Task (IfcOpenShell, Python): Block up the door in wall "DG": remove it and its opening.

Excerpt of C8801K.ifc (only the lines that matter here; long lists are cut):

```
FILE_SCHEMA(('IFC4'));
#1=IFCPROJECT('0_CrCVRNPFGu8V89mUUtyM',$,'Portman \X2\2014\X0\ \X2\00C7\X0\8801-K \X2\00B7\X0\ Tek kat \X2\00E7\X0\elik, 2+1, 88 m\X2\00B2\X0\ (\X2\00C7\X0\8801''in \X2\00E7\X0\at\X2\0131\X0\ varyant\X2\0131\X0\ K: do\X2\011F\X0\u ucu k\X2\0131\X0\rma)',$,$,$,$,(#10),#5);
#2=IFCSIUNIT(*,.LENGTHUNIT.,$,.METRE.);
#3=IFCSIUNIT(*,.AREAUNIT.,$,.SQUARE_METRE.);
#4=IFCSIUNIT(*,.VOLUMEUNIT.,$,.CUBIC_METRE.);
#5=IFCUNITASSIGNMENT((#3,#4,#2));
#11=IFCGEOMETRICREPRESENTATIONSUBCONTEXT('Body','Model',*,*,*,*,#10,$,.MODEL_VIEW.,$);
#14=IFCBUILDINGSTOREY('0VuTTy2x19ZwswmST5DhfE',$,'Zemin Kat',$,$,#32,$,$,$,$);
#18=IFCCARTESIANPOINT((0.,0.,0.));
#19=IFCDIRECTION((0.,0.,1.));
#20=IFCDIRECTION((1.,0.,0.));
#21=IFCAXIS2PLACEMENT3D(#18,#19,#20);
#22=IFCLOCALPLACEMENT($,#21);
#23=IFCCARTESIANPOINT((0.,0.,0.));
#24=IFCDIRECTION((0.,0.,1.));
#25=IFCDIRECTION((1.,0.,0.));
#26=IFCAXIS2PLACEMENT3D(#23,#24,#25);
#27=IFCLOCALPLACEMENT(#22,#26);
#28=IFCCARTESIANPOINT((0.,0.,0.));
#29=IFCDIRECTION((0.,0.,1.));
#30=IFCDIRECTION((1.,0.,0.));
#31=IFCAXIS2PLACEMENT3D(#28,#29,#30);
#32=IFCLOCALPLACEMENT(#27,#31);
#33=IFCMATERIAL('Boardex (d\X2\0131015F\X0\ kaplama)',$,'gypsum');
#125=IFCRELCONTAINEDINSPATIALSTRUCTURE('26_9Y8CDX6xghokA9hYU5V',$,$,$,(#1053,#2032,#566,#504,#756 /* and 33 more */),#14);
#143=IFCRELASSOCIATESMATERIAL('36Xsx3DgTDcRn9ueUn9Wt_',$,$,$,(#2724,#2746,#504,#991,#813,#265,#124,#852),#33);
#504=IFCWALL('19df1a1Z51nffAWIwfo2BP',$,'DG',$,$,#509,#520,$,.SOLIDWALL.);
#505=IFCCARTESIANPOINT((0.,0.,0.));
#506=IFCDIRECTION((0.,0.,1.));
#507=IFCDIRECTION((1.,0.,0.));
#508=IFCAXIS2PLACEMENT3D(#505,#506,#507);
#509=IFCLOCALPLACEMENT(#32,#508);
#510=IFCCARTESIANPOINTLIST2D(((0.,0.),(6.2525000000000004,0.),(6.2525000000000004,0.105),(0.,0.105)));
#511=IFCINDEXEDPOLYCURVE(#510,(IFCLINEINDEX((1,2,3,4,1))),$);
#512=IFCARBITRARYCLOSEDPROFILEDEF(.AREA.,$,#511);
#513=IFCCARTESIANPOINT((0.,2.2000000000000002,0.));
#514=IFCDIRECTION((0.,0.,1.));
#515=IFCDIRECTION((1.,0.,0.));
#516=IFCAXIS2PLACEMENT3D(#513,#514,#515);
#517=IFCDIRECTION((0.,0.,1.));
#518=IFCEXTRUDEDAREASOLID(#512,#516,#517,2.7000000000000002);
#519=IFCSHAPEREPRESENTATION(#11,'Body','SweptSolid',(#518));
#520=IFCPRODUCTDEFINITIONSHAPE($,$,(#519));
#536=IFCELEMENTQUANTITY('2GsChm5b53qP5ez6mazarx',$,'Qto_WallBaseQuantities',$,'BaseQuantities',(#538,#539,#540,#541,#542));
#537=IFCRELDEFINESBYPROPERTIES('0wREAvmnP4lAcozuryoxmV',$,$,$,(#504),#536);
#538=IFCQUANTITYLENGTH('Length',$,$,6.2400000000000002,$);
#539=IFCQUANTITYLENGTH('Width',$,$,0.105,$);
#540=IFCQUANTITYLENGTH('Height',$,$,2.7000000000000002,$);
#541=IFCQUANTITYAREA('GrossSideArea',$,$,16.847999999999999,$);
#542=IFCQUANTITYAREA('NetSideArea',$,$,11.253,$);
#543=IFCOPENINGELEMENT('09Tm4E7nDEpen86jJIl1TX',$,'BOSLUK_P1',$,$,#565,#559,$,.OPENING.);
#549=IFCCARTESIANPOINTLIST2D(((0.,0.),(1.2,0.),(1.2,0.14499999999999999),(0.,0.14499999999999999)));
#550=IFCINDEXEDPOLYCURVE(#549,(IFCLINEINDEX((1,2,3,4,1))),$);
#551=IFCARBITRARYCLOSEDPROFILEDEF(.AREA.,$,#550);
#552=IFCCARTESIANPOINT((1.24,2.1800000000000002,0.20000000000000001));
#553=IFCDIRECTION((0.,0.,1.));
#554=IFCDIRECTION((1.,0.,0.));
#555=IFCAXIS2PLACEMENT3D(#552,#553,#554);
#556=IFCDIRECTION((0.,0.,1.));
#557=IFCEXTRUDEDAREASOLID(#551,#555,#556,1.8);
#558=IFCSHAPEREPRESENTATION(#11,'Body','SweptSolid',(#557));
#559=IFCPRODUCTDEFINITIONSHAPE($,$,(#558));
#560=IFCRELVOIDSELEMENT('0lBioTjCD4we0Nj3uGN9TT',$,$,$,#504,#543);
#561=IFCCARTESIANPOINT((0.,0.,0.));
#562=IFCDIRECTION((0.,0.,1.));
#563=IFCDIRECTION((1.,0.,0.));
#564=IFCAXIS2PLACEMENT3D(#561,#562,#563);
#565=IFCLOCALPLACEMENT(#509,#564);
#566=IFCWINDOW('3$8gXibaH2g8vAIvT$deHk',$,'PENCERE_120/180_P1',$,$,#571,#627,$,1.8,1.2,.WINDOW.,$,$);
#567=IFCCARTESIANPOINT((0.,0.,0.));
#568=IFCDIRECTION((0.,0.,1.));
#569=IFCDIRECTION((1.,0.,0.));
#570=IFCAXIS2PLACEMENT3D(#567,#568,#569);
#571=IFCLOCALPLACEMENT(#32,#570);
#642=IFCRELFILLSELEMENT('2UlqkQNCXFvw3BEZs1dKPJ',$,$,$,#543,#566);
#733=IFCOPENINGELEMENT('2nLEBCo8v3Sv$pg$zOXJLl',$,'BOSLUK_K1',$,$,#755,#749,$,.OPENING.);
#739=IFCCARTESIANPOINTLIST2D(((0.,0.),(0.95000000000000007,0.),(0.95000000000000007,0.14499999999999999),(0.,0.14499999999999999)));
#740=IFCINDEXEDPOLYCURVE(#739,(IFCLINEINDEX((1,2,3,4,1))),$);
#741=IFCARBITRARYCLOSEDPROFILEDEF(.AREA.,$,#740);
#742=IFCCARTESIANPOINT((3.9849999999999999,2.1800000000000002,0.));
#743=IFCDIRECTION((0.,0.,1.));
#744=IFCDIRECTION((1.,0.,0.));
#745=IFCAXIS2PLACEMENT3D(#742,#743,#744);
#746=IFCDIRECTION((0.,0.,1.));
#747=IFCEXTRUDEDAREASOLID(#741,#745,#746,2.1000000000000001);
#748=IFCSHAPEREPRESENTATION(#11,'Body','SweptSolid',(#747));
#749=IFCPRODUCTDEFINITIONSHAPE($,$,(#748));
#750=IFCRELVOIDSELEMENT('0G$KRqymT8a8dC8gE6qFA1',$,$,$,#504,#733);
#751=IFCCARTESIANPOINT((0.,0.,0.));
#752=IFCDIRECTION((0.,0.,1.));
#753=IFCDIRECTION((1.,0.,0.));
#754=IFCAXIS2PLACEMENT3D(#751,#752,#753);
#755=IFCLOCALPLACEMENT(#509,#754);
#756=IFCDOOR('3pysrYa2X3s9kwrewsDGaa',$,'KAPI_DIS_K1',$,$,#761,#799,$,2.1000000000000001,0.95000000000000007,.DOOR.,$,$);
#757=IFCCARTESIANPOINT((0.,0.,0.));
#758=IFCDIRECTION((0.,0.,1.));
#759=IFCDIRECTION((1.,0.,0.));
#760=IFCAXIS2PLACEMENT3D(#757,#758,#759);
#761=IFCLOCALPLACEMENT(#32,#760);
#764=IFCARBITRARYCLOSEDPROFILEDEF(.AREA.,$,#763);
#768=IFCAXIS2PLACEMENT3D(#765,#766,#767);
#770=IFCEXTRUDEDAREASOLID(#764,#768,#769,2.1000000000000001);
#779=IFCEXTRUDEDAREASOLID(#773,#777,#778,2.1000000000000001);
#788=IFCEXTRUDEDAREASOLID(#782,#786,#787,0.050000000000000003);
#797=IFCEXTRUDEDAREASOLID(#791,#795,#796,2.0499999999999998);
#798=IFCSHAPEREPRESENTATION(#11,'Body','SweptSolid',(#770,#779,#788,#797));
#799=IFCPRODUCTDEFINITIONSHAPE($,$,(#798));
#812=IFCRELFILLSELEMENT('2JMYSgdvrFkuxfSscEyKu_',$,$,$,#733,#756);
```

```python
import ifcopenshell
import ifcopenshell.api.feature
import ifcopenshell.api.pset
import ifcopenshell.api.root
import ifcopenshell.geom
import ifcopenshell.util.element
import ifcopenshell.util.shape
import ifcopenshell.util.unit

model = ifcopenshell.open("C8801K.ifc")
area_scale = ifcopenshell.util.unit.calculate_unit_scale(model, "AREAUNIT")
settings = ifcopenshell.geom.settings()


def volume(element):
    """Net volume in cubic metres, openings subtracted."""
    shape = ifcopenshell.geom.create_shape(settings, element)
    return ifcopenshell.util.shape.get_volume(shape.geometry)


door = model.by_id(756)
opening = door.FillsVoids[0].RelatingOpeningElement
wall = opening.VoidsElements[0].RelatingBuildingElement
before = volume(wall)

ifcopenshell.api.root.remove_product(model, product=door)
ifcopenshell.api.feature.remove_feature(model, feature=opening)

after = volume(wall)
thickness = 0.105  # wall thickness in metres

# Update the wall's stored quantities.
qto = model.by_id(ifcopenshell.util.element.get_pset(wall, "Qto_WallBaseQuantities", should_inherit=False)["id"])
ifcopenshell.api.pset.edit_qto(model, qto=qto, properties={"NetSideArea": after / thickness / area_scale})

print(f"wall volume {before:.3f} -> {after:.3f} m3")

model.write("C8801K-out.ifc")
```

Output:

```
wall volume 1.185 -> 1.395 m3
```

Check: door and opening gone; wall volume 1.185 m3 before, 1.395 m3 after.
